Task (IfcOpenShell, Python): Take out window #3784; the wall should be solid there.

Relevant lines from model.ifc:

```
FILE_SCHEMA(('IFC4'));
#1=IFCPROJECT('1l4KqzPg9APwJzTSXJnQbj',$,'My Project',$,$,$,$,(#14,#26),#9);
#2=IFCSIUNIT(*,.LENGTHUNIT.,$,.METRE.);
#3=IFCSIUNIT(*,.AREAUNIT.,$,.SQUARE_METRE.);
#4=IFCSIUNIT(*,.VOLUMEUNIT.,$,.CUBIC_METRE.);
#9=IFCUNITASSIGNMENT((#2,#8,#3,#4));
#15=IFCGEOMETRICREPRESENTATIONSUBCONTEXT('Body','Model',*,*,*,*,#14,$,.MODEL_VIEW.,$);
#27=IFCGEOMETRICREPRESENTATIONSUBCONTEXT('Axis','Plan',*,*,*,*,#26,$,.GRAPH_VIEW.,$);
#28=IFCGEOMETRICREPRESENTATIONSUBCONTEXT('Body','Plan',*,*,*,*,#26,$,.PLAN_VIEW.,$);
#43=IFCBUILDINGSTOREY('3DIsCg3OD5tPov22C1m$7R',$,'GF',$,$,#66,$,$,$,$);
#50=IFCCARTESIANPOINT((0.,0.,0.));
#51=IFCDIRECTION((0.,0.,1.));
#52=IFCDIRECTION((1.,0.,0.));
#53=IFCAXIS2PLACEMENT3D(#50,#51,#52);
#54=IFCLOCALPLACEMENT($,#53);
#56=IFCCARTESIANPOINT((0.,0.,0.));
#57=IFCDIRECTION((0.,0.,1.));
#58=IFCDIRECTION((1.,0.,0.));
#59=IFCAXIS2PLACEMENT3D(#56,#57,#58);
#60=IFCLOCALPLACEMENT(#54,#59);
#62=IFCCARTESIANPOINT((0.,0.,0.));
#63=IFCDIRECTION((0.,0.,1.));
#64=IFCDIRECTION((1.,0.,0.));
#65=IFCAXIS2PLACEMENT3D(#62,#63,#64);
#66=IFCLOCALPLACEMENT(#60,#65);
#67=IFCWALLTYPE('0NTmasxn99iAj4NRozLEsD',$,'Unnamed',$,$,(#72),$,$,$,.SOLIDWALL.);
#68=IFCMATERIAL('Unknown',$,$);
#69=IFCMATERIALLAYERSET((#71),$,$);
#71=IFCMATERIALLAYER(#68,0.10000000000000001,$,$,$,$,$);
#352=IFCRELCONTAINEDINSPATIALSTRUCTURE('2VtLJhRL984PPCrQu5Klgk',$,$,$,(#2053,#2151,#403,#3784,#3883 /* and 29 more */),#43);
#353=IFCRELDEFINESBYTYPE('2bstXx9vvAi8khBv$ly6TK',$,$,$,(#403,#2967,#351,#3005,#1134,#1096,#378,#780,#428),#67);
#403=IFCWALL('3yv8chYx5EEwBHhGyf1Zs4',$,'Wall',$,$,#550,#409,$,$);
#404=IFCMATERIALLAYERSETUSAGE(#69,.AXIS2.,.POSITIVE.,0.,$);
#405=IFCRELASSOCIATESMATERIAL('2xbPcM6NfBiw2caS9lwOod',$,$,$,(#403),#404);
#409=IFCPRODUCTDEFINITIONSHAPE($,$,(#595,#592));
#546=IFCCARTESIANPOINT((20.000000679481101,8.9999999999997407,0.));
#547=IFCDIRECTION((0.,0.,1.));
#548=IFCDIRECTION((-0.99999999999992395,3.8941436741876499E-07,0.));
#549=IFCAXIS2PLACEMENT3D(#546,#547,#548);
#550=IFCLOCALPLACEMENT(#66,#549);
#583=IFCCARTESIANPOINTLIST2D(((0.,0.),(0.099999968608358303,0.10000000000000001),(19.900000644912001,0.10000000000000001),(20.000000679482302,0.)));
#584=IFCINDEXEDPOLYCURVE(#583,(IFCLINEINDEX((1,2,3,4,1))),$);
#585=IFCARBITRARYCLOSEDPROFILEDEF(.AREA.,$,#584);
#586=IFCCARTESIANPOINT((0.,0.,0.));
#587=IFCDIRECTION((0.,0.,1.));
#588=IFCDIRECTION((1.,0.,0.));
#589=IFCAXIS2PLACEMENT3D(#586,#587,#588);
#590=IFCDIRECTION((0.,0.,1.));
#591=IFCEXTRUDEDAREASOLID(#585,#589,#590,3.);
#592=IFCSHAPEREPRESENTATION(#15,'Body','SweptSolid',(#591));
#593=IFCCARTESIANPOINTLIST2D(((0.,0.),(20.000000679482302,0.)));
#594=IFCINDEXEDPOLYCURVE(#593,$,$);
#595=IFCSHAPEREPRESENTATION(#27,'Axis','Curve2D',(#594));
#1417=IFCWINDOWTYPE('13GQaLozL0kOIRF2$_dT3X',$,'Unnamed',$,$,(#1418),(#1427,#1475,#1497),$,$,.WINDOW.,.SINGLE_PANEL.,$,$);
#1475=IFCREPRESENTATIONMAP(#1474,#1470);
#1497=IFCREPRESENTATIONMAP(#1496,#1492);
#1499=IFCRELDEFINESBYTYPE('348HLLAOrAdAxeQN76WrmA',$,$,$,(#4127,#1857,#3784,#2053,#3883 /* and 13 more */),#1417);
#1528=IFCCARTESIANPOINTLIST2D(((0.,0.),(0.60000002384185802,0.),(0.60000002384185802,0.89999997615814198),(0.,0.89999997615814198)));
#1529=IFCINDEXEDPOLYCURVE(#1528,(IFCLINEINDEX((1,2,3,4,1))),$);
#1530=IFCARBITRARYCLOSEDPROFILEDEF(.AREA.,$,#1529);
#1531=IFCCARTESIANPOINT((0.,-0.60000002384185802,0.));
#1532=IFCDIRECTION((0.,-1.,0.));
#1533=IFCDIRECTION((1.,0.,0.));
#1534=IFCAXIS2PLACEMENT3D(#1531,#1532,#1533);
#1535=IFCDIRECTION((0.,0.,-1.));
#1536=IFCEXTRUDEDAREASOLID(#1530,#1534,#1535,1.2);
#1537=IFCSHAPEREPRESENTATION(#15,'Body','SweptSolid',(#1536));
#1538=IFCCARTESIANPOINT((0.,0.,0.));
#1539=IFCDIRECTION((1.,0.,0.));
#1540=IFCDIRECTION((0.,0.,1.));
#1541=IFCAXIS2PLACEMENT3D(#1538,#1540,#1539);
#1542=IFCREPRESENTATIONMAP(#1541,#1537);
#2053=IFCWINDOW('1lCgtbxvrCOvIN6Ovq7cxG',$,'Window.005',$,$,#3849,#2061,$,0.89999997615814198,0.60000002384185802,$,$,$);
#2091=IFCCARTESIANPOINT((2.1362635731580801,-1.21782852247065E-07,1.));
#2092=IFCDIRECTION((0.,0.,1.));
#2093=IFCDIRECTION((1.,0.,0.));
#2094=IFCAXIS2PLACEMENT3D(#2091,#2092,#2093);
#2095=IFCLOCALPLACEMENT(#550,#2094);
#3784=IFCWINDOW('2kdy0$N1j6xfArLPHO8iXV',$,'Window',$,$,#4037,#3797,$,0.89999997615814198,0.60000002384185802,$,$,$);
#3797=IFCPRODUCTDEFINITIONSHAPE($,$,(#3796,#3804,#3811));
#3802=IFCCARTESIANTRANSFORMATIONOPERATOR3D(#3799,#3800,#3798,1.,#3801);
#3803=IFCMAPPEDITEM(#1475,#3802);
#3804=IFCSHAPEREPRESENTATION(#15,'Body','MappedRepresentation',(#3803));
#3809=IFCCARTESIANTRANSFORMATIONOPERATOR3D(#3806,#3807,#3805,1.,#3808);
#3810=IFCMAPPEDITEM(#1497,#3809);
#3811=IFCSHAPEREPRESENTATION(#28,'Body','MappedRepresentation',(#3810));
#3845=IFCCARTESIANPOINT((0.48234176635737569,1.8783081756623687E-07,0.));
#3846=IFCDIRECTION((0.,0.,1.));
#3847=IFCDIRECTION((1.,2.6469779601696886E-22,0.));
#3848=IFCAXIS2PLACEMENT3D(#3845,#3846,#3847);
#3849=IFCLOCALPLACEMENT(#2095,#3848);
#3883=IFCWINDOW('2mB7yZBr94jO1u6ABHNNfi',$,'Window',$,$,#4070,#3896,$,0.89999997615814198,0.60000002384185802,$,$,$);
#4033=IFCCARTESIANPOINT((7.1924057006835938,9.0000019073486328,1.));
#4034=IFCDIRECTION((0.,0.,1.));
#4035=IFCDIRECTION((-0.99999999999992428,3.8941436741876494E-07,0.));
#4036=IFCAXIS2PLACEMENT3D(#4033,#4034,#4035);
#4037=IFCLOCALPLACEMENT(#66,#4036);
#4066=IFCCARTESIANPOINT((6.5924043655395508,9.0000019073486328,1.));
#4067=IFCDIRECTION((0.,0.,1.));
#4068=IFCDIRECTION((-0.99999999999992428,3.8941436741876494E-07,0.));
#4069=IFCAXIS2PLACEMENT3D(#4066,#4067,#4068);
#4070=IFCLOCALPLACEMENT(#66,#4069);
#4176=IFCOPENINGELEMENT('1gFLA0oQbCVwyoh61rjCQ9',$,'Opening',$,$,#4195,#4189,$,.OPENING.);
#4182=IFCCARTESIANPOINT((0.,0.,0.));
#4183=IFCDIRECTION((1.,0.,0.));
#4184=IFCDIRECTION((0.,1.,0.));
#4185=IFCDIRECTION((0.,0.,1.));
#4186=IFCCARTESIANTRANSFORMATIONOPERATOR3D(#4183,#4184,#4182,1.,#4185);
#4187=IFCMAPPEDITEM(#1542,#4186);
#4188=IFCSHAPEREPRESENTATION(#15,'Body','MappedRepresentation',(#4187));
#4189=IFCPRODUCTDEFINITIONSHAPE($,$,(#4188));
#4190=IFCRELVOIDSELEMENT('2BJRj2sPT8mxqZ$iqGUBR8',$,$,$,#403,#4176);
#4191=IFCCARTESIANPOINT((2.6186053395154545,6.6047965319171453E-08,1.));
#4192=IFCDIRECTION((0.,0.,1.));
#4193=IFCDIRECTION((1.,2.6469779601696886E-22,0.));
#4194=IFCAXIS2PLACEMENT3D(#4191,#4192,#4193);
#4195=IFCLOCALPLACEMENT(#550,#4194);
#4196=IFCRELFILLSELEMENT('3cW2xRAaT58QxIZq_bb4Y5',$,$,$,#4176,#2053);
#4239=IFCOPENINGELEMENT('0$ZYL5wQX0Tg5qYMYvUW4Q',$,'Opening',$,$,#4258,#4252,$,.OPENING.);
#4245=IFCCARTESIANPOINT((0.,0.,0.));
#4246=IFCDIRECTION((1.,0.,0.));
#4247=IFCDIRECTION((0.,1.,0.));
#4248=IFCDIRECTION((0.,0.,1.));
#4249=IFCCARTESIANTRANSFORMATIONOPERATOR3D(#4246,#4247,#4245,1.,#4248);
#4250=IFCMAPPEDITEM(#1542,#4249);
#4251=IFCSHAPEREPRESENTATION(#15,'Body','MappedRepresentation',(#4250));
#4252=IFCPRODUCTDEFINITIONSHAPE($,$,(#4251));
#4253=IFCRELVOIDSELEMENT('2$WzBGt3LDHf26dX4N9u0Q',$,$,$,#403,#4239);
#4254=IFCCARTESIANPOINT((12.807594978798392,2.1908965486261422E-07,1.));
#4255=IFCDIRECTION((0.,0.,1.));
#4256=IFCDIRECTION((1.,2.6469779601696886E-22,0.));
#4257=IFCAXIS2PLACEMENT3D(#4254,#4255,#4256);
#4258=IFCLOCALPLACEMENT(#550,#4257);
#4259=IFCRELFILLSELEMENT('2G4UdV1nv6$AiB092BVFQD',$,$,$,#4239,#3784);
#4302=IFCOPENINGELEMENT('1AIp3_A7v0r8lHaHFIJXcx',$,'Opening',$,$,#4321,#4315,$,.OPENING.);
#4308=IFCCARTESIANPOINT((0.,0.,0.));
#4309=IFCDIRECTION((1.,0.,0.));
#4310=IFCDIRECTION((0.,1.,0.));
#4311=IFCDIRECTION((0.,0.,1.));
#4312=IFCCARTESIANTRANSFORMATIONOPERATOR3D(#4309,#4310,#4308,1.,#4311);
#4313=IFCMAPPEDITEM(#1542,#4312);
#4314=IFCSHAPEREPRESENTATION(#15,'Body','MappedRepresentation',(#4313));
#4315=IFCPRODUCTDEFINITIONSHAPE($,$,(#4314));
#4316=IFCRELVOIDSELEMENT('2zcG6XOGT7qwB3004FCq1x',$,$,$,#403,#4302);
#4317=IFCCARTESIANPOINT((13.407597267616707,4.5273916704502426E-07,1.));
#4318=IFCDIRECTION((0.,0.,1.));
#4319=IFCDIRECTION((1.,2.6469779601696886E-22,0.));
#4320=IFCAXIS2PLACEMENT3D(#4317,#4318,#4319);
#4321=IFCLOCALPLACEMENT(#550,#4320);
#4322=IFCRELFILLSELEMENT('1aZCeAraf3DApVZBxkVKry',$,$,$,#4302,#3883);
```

```python
import ifcopenshell
import ifcopenshell.api.feature
import ifcopenshell.api.root
import ifcopenshell.geom
import ifcopenshell.util.shape

model = ifcopenshell.open("model.ifc")
settings = ifcopenshell.geom.settings()


def volume(element):
    """Net volume in cubic metres, openings subtracted."""
    shape = ifcopenshell.geom.create_shape(settings, element)
    return ifcopenshell.util.shape.get_volume(shape.geometry)


window = model.by_guid("2kdy0$N1j6xfArLPHO8iXV")
opening = window.FillsVoids[0].RelatingOpeningElement
wall = opening.VoidsElements[0].RelatingBuildingElement
before = volume(wall)

ifcopenshell.api.root.remove_product(model, product=window)
ifcopenshell.api.feature.remove_feature(model, feature=opening)

after = volume(wall)

print(f"wall volume {before:.3f} -> {after:.3f} m3")

model.write("model_edited.ifc")
```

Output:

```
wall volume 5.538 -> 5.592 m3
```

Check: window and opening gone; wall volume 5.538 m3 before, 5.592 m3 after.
